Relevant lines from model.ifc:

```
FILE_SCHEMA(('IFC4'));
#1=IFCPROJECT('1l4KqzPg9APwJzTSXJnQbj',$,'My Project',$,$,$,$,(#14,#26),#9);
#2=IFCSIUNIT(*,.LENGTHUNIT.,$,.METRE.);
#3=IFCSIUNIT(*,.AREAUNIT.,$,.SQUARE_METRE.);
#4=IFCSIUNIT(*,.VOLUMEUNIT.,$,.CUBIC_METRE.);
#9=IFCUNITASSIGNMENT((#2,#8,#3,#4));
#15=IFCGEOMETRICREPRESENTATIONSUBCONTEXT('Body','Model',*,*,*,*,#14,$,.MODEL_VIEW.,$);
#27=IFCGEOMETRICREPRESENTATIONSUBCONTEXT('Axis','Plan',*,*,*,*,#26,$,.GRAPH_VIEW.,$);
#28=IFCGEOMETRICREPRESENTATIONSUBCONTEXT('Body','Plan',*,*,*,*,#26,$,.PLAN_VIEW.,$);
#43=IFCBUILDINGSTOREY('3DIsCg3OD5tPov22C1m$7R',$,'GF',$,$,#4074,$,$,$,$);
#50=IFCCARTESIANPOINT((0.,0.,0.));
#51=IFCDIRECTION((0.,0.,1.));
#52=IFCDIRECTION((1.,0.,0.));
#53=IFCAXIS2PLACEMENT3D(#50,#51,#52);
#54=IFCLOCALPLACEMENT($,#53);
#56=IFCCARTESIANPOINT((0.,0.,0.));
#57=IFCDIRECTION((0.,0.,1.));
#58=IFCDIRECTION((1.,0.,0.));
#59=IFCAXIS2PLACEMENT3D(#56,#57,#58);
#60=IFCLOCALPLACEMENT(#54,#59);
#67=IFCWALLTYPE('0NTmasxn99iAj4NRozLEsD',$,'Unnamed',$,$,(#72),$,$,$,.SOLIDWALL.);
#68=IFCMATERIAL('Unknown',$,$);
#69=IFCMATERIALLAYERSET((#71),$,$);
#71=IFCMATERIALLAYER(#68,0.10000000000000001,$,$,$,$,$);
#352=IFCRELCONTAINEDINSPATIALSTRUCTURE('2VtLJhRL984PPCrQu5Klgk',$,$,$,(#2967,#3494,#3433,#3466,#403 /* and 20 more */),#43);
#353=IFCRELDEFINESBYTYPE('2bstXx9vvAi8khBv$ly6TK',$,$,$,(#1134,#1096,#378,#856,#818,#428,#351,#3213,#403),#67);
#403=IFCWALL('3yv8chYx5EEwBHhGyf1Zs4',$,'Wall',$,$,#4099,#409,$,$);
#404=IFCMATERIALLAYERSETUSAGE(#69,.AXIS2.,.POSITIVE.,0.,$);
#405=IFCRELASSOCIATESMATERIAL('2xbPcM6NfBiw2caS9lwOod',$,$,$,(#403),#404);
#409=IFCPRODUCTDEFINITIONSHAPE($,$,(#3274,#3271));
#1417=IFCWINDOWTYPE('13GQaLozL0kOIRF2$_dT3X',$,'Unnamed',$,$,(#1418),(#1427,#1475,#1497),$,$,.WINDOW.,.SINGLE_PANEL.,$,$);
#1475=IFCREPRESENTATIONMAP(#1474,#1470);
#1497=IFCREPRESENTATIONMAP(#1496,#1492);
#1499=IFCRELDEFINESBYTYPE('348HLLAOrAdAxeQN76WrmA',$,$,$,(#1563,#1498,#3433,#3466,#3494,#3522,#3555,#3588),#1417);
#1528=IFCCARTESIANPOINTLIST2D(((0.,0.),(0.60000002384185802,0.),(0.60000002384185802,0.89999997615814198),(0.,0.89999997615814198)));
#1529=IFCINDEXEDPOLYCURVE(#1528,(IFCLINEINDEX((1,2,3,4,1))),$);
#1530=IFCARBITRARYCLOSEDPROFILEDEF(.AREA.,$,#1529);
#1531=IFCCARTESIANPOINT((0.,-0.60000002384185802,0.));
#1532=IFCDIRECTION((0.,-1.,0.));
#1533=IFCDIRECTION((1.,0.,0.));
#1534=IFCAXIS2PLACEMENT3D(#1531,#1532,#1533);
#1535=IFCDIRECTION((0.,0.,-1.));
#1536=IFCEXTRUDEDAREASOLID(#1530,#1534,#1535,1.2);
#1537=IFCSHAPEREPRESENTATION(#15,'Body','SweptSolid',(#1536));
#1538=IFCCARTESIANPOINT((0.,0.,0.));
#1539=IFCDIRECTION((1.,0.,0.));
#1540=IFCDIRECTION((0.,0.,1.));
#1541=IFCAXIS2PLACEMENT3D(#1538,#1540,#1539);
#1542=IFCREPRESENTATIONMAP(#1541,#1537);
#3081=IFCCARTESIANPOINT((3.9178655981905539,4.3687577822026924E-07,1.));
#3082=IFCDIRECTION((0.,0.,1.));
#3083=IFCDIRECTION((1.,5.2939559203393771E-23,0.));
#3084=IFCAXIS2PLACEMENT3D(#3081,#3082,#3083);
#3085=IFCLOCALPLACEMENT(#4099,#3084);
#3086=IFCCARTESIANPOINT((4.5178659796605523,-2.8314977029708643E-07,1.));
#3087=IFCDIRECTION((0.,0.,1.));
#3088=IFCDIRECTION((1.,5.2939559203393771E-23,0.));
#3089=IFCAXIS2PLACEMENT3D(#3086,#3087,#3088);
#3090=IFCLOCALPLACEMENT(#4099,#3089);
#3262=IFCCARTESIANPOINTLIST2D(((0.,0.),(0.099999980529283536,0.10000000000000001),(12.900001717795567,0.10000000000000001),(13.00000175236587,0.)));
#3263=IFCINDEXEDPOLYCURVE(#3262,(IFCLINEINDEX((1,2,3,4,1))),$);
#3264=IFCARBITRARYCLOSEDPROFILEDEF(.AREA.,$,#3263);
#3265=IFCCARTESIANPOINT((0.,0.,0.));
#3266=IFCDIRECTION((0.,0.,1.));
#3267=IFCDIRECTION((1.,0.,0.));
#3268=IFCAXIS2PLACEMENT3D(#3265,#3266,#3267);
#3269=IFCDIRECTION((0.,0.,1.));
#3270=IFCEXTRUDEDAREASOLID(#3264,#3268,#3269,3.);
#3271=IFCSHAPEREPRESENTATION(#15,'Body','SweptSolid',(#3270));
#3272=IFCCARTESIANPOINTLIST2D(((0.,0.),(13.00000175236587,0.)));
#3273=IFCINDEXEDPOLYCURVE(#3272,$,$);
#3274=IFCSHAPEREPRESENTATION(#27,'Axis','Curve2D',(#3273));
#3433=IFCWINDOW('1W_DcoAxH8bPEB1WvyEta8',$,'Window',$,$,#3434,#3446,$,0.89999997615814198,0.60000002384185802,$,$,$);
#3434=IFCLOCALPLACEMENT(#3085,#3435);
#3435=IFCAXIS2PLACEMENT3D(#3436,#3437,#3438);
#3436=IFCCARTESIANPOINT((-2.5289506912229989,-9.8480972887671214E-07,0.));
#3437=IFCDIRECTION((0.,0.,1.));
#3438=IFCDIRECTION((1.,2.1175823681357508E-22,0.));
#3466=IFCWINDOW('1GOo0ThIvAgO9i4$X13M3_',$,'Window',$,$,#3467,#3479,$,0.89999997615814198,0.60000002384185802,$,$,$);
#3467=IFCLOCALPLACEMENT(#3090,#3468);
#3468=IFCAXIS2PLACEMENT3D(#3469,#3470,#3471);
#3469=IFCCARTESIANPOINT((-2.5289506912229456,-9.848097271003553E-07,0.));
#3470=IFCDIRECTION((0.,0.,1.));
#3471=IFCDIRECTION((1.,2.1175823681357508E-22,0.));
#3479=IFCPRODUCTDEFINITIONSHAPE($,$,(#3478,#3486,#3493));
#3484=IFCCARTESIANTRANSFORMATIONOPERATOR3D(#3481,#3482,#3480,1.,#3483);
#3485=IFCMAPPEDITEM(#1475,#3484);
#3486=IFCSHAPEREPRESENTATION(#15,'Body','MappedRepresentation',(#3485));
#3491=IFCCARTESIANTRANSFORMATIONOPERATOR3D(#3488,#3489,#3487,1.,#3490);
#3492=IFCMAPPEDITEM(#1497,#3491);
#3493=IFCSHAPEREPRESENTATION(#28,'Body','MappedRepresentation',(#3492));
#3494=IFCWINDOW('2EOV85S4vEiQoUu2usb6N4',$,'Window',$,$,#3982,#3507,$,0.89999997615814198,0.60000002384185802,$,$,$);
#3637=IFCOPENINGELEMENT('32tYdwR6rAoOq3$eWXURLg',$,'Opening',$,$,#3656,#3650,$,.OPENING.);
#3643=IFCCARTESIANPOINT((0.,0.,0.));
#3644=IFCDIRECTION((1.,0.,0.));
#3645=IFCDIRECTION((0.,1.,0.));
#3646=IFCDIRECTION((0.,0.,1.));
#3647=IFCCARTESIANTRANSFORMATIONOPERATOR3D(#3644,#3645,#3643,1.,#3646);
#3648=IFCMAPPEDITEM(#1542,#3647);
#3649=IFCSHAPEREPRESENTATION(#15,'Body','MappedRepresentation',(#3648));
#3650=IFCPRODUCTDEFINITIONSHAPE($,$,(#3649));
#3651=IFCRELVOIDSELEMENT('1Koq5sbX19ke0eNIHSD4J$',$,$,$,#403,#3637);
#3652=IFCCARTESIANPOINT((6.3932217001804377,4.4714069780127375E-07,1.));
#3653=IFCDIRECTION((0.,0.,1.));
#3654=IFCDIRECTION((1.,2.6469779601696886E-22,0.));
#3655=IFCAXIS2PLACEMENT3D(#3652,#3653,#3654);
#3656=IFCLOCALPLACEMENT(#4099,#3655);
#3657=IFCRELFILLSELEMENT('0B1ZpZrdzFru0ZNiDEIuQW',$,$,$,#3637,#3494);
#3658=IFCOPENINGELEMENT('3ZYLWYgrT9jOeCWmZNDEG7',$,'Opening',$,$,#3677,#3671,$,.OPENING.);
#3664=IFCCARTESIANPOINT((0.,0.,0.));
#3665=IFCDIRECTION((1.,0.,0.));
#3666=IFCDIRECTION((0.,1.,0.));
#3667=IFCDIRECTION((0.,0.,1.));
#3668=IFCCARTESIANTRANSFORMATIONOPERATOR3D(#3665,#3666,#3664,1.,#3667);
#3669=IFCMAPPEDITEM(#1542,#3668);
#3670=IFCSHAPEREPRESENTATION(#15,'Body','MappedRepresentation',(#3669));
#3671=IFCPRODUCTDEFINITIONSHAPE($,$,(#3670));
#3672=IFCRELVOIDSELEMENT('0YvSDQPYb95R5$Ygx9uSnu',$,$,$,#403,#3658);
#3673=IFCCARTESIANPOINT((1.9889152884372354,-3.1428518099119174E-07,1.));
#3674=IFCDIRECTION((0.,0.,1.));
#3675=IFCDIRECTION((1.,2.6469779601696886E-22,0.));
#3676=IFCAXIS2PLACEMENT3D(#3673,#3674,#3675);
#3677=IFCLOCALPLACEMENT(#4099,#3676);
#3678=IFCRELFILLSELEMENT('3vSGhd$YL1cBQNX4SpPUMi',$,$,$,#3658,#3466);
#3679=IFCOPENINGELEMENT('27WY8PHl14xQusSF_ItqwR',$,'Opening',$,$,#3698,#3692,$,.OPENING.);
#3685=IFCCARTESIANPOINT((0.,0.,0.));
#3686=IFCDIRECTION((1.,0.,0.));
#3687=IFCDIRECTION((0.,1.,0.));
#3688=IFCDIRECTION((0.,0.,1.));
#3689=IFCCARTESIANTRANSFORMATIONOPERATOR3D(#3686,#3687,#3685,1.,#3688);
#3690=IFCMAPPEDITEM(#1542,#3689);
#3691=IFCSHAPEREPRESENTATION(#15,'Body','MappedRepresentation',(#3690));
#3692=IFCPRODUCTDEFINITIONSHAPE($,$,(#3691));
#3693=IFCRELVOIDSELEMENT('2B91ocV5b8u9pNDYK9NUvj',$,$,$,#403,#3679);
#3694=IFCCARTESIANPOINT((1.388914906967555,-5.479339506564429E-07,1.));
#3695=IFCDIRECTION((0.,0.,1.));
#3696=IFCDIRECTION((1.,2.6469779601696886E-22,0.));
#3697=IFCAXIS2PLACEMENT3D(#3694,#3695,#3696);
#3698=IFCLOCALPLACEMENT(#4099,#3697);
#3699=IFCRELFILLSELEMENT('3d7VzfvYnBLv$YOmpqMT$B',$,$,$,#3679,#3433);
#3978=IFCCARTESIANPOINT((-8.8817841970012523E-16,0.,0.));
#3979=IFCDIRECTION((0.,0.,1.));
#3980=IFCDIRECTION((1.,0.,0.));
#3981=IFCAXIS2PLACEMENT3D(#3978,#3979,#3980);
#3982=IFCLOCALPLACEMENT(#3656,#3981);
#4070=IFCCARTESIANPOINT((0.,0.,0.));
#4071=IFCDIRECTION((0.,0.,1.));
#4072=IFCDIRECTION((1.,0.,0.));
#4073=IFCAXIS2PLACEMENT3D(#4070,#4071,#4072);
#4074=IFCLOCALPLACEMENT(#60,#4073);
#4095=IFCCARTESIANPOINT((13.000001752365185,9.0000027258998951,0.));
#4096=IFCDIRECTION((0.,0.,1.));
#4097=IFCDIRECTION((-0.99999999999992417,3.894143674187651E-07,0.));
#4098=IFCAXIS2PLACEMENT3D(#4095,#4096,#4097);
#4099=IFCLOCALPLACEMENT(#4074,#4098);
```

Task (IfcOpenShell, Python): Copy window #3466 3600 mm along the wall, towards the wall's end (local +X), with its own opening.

```python
import ifcopenshell
import ifcopenshell.api.feature
import ifcopenshell.api.geometry
import ifcopenshell.api.root
import ifcopenshell.geom
import ifcopenshell.util.element
import ifcopenshell.util.placement
import ifcopenshell.util.shape
import ifcopenshell.util.unit

model = ifcopenshell.open("model.ifc")
unit_scale = ifcopenshell.util.unit.calculate_unit_scale(model)
settings = ifcopenshell.geom.settings()


def volume(element):
    """Net volume in cubic metres, openings subtracted."""
    shape = ifcopenshell.geom.create_shape(settings, element)
    return ifcopenshell.util.shape.get_volume(shape.geometry)


window = model.by_guid("1GOo0ThIvAgO9i4$X13M3_")
opening = window.FillsVoids[0].RelatingOpeningElement
wall = opening.VoidsElements[0].RelatingBuildingElement
before = volume(wall)
shift = ifcopenshell.util.placement.get_local_placement(wall.ObjectPlacement)[:3, 0] * 3.6 / unit_scale

# copy_class copies the void relationship, type, container and properties, but no geometry.
new_opening = ifcopenshell.api.root.copy_class(model, product=opening)
new_opening.Representation = ifcopenshell.util.element.copy_deep(
    model, opening.Representation, exclude=["IfcGeometricRepresentationContext", "IfcRepresentationMap"]
)
new_window = ifcopenshell.api.root.copy_class(model, product=window)
new_window.Representation = ifcopenshell.util.element.copy_deep(
    model, window.Representation, exclude=["IfcGeometricRepresentationContext", "IfcRepresentationMap"]
)
ifcopenshell.api.feature.add_filling(model, opening=new_opening, element=new_window)

for old, new in ((opening, new_opening), (window, new_window)):
    matrix = ifcopenshell.util.placement.get_local_placement(old.ObjectPlacement)
    matrix[:3, 3] += shift
    ifcopenshell.api.geometry.edit_object_placement(model, product=new, matrix=matrix, is_si=False)

after = volume(wall)

print(f"wall volume {before:.3f} -> {after:.3f} m3")

model.write("model_edited.ifc")
```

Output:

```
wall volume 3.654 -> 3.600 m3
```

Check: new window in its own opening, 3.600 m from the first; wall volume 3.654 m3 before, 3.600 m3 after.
